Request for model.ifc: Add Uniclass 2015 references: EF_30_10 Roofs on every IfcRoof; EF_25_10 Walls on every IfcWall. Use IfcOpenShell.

First a look at what the model holds.

```python
import ifcopenshell

model = ifcopenshell.open("model.ifc")
print(model.schema)
print("classifications:", [c.Name for c in model.by_type("IfcClassification")])
for ifc_class in ("IfcDoor", "IfcRoof", "IfcStair", "IfcWall", "IfcWindow"):
    print(ifc_class, len(model.by_type(ifc_class)))
```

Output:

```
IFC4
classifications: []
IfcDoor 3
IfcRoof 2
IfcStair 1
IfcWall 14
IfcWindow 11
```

```python
import ifcopenshell
import ifcopenshell.api.classification

model = ifcopenshell.open("model.ifc")

system = ifcopenshell.api.classification.add_classification(model, classification="Uniclass 2015")

codes = {
    "IfcRoof": ("EF_30_10", "Roofs"),
    "IfcWall": ("EF_25_10", "Walls"),
}
for ifc_class, (code, name) in codes.items():
    products = model.by_type(ifc_class)
    ifcopenshell.api.classification.add_reference(
        model, products=products, classification=system, identification=code, name=name
    )
    print(code, len(products))

model.write("model-out.ifc")
```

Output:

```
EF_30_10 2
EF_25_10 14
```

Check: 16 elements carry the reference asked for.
